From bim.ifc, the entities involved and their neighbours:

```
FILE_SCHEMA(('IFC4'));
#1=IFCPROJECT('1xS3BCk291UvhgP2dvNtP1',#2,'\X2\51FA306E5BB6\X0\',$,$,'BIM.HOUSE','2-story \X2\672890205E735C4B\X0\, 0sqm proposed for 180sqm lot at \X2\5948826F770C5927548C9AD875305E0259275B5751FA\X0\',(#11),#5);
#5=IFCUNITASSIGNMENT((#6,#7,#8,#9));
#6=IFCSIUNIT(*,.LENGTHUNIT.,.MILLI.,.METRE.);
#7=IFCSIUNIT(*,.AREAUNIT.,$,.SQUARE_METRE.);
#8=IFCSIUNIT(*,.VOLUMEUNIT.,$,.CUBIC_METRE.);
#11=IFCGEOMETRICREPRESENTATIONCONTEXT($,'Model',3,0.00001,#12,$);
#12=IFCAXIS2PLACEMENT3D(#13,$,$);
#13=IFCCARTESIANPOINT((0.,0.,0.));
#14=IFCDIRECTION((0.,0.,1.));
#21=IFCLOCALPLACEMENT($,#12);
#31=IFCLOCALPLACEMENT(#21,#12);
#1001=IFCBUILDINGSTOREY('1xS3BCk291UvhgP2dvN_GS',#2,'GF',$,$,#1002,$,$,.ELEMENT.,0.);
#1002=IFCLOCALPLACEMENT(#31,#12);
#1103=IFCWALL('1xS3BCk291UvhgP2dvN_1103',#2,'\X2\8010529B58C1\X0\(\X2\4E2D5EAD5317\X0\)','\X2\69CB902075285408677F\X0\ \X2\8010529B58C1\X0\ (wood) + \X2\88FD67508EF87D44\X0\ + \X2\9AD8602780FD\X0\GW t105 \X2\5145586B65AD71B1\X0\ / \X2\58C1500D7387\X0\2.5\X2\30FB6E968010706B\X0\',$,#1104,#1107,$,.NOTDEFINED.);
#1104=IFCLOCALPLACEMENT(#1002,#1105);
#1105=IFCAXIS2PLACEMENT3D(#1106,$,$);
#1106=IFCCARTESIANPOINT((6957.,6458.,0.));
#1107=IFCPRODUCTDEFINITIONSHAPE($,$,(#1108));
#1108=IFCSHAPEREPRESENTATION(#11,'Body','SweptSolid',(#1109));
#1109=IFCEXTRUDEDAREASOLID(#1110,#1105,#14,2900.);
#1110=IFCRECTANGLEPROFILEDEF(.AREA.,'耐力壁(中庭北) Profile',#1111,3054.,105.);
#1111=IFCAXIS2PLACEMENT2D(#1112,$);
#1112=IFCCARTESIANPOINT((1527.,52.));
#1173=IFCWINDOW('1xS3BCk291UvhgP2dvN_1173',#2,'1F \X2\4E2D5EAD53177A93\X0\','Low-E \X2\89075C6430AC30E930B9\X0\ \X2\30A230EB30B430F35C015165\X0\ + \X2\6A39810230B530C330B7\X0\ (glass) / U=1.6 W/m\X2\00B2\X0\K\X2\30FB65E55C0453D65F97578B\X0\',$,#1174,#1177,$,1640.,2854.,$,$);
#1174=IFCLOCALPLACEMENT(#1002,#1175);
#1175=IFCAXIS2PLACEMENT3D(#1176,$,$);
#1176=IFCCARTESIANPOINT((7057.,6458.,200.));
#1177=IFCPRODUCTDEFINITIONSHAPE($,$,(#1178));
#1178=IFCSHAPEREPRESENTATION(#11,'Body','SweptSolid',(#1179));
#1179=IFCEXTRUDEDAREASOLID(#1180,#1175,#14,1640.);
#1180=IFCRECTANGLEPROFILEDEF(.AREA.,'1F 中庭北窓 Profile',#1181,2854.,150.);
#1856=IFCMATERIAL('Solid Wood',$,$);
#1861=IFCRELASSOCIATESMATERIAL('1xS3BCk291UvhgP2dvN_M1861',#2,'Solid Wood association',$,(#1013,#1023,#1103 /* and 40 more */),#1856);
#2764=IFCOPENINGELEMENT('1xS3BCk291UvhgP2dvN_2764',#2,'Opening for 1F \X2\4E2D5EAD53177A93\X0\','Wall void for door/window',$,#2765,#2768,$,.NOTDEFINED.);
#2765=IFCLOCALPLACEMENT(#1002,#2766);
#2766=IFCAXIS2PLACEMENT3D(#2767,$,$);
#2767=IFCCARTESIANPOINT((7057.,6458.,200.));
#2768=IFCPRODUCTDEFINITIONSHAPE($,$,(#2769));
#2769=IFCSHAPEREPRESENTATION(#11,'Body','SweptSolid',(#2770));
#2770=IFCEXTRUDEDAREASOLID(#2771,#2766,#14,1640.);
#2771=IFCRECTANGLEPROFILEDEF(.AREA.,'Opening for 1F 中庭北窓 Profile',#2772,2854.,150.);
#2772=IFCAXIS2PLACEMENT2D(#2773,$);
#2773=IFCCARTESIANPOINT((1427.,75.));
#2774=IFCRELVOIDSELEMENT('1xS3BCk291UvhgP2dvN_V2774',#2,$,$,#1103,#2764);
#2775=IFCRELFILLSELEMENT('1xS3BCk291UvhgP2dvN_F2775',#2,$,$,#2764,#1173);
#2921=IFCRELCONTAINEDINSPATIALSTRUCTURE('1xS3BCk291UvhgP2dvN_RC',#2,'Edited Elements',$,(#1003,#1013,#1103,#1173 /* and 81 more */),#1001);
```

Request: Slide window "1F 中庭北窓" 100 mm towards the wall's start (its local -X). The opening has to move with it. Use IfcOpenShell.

```python
import ifcopenshell
import ifcopenshell.api.geometry
import ifcopenshell.util.placement
import ifcopenshell.util.unit

model = ifcopenshell.open("bim.ifc")
unit_scale = ifcopenshell.util.unit.calculate_unit_scale(model)

window = model.by_id(1173)
opening = window.FillsVoids[0].RelatingOpeningElement
wall = opening.VoidsElements[0].RelatingBuildingElement

wall_matrix = ifcopenshell.util.placement.get_local_placement(wall.ObjectPlacement)
shift = wall_matrix[:3, 0] * -0.1 / unit_scale
before = ifcopenshell.util.placement.get_local_placement(window.ObjectPlacement)[:3, 3].copy()

# The window is not placed relative to its opening, so move both.
for product in (opening, window):
    matrix = ifcopenshell.util.placement.get_local_placement(product.ObjectPlacement)
    matrix[:3, 3] += shift
    ifcopenshell.api.geometry.edit_object_placement(model, product=product, matrix=matrix, is_si=False)

after = ifcopenshell.util.placement.get_local_placement(window.ObjectPlacement)[:3, 3]
print("window moved by", (after - before).round(3) + 0.0)

model.write("bim_v2.ifc")
```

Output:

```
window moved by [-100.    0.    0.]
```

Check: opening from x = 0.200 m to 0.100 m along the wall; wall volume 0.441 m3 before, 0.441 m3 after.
